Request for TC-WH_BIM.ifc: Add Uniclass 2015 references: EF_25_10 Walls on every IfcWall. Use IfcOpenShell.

First a look at what the model holds.

```python
import ifcopenshell

model = ifcopenshell.open("TC-WH_BIM.ifc")
print(model.schema)
print("classifications:", [c.Name for c in model.by_type("IfcClassification")])
for ifc_class in ("IfcDoor", "IfcRoof", "IfcStair", "IfcWall", "IfcWindow"):
    print(ifc_class, len(model.by_type(ifc_class)))
```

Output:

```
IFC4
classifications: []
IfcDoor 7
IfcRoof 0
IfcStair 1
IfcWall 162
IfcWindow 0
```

```python
import ifcopenshell
import ifcopenshell.api.classification

model = ifcopenshell.open("TC-WH_BIM.ifc")

system = ifcopenshell.api.classification.add_classification(model, classification="Uniclass 2015")

codes = {
    "IfcWall": ("EF_25_10", "Walls"),
}
for ifc_class, (code, name) in codes.items():
    products = model.by_type(ifc_class)
    ifcopenshell.api.classification.add_reference(
        model, products=products, classification=system, identification=code, name=name
    )
    print(code, len(products))

model.write("TC-WH_BIM-out.ifc")
```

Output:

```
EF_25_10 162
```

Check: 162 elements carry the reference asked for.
